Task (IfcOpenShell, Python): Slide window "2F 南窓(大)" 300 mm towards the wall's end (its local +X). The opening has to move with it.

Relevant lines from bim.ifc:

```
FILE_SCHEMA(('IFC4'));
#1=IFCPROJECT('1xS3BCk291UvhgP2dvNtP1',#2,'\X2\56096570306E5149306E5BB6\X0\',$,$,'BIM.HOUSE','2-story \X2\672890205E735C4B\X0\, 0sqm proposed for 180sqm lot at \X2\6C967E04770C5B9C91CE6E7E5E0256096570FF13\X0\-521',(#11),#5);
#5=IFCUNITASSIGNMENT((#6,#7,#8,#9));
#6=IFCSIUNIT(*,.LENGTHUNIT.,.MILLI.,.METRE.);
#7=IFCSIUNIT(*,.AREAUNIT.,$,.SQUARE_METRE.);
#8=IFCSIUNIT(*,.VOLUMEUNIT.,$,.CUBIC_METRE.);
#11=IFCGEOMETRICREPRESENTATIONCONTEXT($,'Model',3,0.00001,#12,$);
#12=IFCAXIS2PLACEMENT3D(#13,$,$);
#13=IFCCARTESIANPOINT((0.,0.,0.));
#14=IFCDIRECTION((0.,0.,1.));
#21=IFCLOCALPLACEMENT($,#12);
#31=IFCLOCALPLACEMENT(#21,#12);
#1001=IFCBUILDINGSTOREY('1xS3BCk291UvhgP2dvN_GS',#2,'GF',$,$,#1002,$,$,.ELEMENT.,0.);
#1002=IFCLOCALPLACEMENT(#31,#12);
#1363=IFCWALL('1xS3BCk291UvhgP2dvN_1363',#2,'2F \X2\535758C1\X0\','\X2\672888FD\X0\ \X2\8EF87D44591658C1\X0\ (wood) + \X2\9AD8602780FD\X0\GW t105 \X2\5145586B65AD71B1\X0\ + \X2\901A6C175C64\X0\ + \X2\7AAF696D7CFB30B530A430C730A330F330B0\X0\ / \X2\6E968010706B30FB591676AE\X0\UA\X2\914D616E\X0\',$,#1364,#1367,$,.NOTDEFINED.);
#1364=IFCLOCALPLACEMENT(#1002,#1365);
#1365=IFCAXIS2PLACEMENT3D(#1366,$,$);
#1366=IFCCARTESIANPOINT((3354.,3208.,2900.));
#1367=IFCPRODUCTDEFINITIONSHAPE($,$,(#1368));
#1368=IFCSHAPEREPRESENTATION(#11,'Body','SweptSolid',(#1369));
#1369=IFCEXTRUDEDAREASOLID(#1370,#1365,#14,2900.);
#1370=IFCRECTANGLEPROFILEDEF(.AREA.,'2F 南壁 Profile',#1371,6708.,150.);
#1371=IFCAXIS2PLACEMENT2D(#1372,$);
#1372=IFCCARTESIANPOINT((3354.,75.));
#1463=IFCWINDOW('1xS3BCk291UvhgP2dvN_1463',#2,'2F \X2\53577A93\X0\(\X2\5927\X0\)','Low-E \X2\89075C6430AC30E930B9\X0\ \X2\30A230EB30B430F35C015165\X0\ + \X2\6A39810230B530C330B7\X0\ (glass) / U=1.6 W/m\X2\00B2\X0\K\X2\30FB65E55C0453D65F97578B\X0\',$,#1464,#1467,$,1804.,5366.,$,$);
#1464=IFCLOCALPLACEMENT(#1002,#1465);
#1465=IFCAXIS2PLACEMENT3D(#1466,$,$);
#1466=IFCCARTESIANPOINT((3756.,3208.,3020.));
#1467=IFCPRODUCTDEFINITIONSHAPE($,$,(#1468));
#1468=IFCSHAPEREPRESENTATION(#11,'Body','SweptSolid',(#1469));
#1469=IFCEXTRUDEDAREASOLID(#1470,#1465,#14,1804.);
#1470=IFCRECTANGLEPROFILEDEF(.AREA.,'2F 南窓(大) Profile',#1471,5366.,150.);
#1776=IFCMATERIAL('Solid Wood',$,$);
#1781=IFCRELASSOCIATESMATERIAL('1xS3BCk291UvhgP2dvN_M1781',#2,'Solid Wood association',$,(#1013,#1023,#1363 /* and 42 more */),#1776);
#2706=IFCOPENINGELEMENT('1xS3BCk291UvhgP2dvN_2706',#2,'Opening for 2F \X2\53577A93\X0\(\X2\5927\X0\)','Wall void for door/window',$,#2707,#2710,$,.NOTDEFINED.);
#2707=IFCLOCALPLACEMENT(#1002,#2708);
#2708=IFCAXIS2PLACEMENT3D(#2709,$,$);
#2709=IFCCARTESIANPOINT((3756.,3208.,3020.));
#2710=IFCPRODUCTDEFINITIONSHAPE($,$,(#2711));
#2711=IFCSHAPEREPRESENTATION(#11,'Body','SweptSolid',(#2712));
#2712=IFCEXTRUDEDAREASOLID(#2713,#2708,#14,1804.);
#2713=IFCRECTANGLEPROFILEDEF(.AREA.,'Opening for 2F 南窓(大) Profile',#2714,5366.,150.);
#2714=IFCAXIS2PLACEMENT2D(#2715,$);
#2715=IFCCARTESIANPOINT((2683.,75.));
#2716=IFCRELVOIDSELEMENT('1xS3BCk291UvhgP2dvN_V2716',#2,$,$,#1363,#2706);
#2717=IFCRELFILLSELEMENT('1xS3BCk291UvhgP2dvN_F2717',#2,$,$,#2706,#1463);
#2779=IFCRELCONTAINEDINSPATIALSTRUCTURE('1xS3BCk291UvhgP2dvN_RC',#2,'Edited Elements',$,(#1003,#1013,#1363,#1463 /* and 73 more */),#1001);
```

```python
import ifcopenshell
import ifcopenshell.api.geometry
import ifcopenshell.util.placement

model = ifcopenshell.open("bim.ifc")

window = model.by_id(1463)
opening = window.FillsVoids[0].RelatingOpeningElement
wall = opening.VoidsElements[0].RelatingBuildingElement

wall_matrix = ifcopenshell.util.placement.get_local_placement(wall.ObjectPlacement)
shift = wall_matrix[:3, 0] * 300.0
before = ifcopenshell.util.placement.get_local_placement(window.ObjectPlacement)[:3, 3].copy()

# The window is not placed relative to its opening, so move both.
for product in (opening, window):
    matrix = ifcopenshell.util.placement.get_local_placement(product.ObjectPlacement)
    matrix[:3, 3] += shift
    ifcopenshell.api.geometry.edit_object_placement(model, product=product, matrix=matrix, is_si=False)

after = ifcopenshell.util.placement.get_local_placement(window.ObjectPlacement)[:3, 3]
print("window moved by", (after - before).round(3) + 0.0)

model.write("bim-out.ifc")
```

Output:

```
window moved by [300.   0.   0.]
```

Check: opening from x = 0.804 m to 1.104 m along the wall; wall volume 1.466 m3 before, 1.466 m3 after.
